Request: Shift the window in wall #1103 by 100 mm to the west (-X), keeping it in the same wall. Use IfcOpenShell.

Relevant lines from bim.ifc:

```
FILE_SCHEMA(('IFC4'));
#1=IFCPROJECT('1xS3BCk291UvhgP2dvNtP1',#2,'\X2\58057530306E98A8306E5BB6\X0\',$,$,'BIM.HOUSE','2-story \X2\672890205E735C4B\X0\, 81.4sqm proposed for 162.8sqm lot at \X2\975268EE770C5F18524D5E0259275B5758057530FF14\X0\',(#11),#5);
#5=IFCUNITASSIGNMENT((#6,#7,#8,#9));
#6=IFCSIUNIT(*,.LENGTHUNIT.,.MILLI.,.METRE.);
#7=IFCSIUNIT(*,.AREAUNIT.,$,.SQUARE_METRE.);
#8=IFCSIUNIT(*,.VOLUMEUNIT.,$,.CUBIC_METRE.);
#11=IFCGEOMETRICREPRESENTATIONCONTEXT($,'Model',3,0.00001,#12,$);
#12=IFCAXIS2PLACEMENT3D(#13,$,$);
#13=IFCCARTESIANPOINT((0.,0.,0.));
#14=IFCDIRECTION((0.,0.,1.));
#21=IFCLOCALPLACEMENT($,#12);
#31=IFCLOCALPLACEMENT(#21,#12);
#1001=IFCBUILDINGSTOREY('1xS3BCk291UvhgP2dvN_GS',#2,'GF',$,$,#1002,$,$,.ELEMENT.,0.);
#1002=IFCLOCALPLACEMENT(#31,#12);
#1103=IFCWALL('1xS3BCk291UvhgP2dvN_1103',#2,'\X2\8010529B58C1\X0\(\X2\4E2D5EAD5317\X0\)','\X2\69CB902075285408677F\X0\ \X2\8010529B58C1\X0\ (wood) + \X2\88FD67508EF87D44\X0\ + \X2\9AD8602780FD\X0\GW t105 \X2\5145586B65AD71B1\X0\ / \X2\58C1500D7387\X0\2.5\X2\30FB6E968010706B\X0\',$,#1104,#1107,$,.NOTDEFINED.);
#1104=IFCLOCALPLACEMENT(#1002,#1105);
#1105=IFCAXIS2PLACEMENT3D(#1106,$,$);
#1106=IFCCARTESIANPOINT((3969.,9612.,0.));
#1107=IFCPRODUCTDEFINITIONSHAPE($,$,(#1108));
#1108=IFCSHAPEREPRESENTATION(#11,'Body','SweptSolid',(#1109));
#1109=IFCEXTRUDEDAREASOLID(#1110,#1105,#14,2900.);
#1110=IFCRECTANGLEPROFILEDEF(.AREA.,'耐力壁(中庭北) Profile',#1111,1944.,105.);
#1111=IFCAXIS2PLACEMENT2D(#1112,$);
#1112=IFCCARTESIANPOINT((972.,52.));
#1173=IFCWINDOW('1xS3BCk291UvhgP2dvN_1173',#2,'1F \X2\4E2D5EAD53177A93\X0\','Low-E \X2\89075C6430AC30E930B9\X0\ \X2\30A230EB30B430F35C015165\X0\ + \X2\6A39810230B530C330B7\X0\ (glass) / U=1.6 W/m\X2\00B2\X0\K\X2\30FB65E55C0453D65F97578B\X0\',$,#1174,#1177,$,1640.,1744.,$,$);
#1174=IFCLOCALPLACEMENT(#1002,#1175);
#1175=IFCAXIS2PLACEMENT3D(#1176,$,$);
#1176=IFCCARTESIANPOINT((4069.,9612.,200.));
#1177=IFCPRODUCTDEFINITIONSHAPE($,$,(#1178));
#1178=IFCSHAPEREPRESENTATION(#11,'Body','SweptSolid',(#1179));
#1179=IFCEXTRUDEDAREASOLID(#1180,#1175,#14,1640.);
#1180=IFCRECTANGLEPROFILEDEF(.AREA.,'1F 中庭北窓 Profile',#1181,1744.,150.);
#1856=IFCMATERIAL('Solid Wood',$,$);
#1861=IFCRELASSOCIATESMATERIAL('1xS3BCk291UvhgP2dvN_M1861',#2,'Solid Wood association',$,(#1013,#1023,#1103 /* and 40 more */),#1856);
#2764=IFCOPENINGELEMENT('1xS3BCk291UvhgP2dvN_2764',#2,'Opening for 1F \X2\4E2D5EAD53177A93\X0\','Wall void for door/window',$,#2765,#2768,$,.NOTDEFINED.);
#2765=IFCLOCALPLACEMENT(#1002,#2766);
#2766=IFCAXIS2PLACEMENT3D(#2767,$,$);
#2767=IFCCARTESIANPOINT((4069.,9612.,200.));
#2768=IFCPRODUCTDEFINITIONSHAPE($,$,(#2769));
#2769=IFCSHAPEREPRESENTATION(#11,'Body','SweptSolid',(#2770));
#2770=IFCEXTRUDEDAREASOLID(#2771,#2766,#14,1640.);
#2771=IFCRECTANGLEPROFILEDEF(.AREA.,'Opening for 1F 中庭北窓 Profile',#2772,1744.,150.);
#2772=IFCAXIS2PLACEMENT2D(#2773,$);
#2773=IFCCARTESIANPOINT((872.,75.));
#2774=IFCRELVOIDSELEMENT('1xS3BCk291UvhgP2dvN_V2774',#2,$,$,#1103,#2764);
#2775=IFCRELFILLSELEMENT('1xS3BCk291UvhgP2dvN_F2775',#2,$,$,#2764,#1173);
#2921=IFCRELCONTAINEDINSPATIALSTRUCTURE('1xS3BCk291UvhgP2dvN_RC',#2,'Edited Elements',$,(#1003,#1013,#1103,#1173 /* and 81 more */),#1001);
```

```python
import ifcopenshell
import ifcopenshell.api.geometry
import ifcopenshell.util.placement

model = ifcopenshell.open("bim.ifc")

window = model.by_guid("1xS3BCk291UvhgP2dvN_1173")
opening = window.FillsVoids[0].RelatingOpeningElement
wall = opening.VoidsElements[0].RelatingBuildingElement

wall_matrix = ifcopenshell.util.placement.get_local_placement(wall.ObjectPlacement)
shift = wall_matrix[:3, 0] * -100.0
before = ifcopenshell.util.placement.get_local_placement(window.ObjectPlacement)[:3, 3].copy()

# The window is not placed relative to its opening, so move both.
for product in (opening, window):
    matrix = ifcopenshell.util.placement.get_local_placement(product.ObjectPlacement)
    matrix[:3, 3] += shift
    ifcopenshell.api.geometry.edit_object_placement(model, product=product, matrix=matrix, is_si=False)

after = ifcopenshell.util.placement.get_local_placement(window.ObjectPlacement)[:3, 3]
print("window moved by", (after - before).round(3) + 0.0)

model.write("bim_updated.ifc")
```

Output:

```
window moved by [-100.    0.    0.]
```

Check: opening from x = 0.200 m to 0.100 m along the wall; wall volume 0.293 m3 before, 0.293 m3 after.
